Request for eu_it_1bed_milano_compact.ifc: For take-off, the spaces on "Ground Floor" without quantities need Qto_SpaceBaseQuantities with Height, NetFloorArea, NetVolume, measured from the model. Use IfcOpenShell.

First a look at what the model holds.

```python
import ifcopenshell
import ifcopenshell.util.element
import ifcopenshell.util.unit

model = ifcopenshell.open("eu_it_1bed_milano_compact.ifc")
print(model.schema)
for unit_type in ("LENGTHUNIT", "AREAUNIT", "VOLUMEUNIT"):
    print(unit_type, ifcopenshell.util.unit.calculate_unit_scale(model, unit_type))
storey = next(s for s in model.by_type("IfcBuildingStorey") if s.Name == "Ground Floor")
spaces = [e for e in ifcopenshell.util.element.get_decomposition(storey) if e.is_a("IfcSpace")]
for e in sorted(spaces, key=lambda e: e.id()):
    print(e.id(), e.is_a(), e.Name, list(ifcopenshell.util.element.get_psets(e, qtos_only=True)), sep=" | ")
```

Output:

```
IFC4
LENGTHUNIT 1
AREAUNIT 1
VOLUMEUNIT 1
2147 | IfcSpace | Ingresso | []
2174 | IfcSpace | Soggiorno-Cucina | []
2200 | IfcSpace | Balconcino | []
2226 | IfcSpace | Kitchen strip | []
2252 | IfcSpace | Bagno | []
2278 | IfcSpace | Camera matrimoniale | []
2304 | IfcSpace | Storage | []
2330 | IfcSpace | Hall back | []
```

```python
import ifcopenshell
import ifcopenshell.api.pset
import ifcopenshell.geom
import ifcopenshell.util.element
import ifcopenshell.util.shape
import ifcopenshell.util.unit

model = ifcopenshell.open("eu_it_1bed_milano_compact.ifc")
unit_scale = ifcopenshell.util.unit.calculate_unit_scale(model)
area_scale = ifcopenshell.util.unit.calculate_unit_scale(model, "AREAUNIT")
volume_scale = ifcopenshell.util.unit.calculate_unit_scale(model, "VOLUMEUNIT")
settings = ifcopenshell.geom.settings()

storey = next(s for s in model.by_type("IfcBuildingStorey") if s.Name == "Ground Floor")
spaces = [e for e in ifcopenshell.util.element.get_decomposition(storey) if e.is_a("IfcSpace")]

for e in sorted(spaces, key=lambda e: e.id()):
    if ifcopenshell.util.element.get_psets(e, qtos_only=True, should_inherit=False):
        continue
    # Geometry comes back in metres, in the element's own axes.
    shape = ifcopenshell.geom.create_shape(settings, e)
    values = {
        "Height": ifcopenshell.util.shape.get_z(shape.geometry) / unit_scale,
        "NetFloorArea": ifcopenshell.util.shape.get_footprint_area(shape.geometry) / area_scale,
        "NetVolume": ifcopenshell.util.shape.get_volume(shape.geometry) / volume_scale,
    }
    qto = ifcopenshell.api.pset.add_qto(model, product=e, name="Qto_SpaceBaseQuantities")
    ifcopenshell.api.pset.edit_qto(model, qto=qto, properties=values)
    print(e.id(), {k: round(v, 3) for k, v in values.items()})

model.write("eu_it_1bed_milano_compact-out.ifc")
```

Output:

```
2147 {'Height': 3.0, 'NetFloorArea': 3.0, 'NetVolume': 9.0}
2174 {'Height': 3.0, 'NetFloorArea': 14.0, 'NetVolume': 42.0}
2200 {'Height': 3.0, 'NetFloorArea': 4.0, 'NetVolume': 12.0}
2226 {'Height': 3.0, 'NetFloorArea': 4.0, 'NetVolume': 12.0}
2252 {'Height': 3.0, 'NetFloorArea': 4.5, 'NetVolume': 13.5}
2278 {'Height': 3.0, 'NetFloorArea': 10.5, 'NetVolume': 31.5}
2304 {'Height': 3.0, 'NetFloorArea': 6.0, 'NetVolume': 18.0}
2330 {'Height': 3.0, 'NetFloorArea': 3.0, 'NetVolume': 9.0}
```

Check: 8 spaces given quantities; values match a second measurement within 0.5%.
